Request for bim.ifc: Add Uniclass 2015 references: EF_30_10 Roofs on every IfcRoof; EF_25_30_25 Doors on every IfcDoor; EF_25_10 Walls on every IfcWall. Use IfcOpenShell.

First a look at what the model holds.

```python
import ifcopenshell

model = ifcopenshell.open("bim.ifc")
print(model.schema)
print("classifications:", [c.Name for c in model.by_type("IfcClassification")])
for ifc_class in ("IfcDoor", "IfcRoof", "IfcStair", "IfcWall", "IfcWindow"):
    print(ifc_class, len(model.by_type(ifc_class)))
```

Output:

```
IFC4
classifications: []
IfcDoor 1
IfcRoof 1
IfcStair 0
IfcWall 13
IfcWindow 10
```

```python
import ifcopenshell
import ifcopenshell.api.classification

model = ifcopenshell.open("bim.ifc")

system = ifcopenshell.api.classification.add_classification(model, classification="Uniclass 2015")

codes = {
    "IfcRoof": ("EF_30_10", "Roofs"),
    "IfcDoor": ("EF_25_30_25", "Doors"),
    "IfcWall": ("EF_25_10", "Walls"),
}
for ifc_class, (code, name) in codes.items():
    products = model.by_type(ifc_class)
    ifcopenshell.api.classification.add_reference(
        model, products=products, classification=system, identification=code, name=name
    )
    print(code, len(products))

model.write("bim_v2.ifc")
```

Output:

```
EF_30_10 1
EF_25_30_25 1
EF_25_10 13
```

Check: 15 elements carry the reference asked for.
